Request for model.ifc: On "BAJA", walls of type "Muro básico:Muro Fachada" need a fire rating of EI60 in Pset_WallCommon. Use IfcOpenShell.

First a look at what the model holds.

```python
import ifcopenshell
import ifcopenshell.util.element

model = ifcopenshell.open("model.ifc")
print(model.schema)
storey = next(s for s in model.by_type("IfcBuildingStorey") if s.Name == "BAJA")
walls = [e for e in ifcopenshell.util.element.get_decomposition(storey) if e.is_a("IfcWall")]
seen = {}
for e in walls:
    element_type = ifcopenshell.util.element.get_type(e)
    key = (element_type.Name if element_type != e and element_type else None, ifcopenshell.util.element.get_pset(e, "Pset_WallCommon", "FireRating"))
    seen[key] = seen.get(key, 0) + 1
for (name, value), count in sorted(seen.items(), key=str):
    print(count, "x", name, "|", value)
```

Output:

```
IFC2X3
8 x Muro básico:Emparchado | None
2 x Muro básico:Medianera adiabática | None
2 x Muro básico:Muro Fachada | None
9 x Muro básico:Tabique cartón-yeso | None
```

```python
import ifcopenshell
import ifcopenshell.api.pset
import ifcopenshell.util.element

model = ifcopenshell.open("model.ifc")

storey = next(s for s in model.by_type("IfcBuildingStorey") if s.Name == "BAJA")
walls = [e for e in ifcopenshell.util.element.get_decomposition(storey) if e.is_a("IfcWall")]

count = 0
for e in walls:
    element_type = ifcopenshell.util.element.get_type(e)
    if element_type in (None, e) or element_type.Name != "Muro básico:Muro Fachada":
        continue
    # add_pset returns the element's existing set when there is one.
    pset = ifcopenshell.api.pset.add_pset(model, product=e, name="Pset_WallCommon")
    ifcopenshell.api.pset.edit_pset(model, pset=pset, properties={"FireRating": "EI60"})
    count += 1

print(count, "walls updated")

model.write("model-out.ifc")
```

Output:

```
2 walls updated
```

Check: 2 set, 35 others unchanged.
